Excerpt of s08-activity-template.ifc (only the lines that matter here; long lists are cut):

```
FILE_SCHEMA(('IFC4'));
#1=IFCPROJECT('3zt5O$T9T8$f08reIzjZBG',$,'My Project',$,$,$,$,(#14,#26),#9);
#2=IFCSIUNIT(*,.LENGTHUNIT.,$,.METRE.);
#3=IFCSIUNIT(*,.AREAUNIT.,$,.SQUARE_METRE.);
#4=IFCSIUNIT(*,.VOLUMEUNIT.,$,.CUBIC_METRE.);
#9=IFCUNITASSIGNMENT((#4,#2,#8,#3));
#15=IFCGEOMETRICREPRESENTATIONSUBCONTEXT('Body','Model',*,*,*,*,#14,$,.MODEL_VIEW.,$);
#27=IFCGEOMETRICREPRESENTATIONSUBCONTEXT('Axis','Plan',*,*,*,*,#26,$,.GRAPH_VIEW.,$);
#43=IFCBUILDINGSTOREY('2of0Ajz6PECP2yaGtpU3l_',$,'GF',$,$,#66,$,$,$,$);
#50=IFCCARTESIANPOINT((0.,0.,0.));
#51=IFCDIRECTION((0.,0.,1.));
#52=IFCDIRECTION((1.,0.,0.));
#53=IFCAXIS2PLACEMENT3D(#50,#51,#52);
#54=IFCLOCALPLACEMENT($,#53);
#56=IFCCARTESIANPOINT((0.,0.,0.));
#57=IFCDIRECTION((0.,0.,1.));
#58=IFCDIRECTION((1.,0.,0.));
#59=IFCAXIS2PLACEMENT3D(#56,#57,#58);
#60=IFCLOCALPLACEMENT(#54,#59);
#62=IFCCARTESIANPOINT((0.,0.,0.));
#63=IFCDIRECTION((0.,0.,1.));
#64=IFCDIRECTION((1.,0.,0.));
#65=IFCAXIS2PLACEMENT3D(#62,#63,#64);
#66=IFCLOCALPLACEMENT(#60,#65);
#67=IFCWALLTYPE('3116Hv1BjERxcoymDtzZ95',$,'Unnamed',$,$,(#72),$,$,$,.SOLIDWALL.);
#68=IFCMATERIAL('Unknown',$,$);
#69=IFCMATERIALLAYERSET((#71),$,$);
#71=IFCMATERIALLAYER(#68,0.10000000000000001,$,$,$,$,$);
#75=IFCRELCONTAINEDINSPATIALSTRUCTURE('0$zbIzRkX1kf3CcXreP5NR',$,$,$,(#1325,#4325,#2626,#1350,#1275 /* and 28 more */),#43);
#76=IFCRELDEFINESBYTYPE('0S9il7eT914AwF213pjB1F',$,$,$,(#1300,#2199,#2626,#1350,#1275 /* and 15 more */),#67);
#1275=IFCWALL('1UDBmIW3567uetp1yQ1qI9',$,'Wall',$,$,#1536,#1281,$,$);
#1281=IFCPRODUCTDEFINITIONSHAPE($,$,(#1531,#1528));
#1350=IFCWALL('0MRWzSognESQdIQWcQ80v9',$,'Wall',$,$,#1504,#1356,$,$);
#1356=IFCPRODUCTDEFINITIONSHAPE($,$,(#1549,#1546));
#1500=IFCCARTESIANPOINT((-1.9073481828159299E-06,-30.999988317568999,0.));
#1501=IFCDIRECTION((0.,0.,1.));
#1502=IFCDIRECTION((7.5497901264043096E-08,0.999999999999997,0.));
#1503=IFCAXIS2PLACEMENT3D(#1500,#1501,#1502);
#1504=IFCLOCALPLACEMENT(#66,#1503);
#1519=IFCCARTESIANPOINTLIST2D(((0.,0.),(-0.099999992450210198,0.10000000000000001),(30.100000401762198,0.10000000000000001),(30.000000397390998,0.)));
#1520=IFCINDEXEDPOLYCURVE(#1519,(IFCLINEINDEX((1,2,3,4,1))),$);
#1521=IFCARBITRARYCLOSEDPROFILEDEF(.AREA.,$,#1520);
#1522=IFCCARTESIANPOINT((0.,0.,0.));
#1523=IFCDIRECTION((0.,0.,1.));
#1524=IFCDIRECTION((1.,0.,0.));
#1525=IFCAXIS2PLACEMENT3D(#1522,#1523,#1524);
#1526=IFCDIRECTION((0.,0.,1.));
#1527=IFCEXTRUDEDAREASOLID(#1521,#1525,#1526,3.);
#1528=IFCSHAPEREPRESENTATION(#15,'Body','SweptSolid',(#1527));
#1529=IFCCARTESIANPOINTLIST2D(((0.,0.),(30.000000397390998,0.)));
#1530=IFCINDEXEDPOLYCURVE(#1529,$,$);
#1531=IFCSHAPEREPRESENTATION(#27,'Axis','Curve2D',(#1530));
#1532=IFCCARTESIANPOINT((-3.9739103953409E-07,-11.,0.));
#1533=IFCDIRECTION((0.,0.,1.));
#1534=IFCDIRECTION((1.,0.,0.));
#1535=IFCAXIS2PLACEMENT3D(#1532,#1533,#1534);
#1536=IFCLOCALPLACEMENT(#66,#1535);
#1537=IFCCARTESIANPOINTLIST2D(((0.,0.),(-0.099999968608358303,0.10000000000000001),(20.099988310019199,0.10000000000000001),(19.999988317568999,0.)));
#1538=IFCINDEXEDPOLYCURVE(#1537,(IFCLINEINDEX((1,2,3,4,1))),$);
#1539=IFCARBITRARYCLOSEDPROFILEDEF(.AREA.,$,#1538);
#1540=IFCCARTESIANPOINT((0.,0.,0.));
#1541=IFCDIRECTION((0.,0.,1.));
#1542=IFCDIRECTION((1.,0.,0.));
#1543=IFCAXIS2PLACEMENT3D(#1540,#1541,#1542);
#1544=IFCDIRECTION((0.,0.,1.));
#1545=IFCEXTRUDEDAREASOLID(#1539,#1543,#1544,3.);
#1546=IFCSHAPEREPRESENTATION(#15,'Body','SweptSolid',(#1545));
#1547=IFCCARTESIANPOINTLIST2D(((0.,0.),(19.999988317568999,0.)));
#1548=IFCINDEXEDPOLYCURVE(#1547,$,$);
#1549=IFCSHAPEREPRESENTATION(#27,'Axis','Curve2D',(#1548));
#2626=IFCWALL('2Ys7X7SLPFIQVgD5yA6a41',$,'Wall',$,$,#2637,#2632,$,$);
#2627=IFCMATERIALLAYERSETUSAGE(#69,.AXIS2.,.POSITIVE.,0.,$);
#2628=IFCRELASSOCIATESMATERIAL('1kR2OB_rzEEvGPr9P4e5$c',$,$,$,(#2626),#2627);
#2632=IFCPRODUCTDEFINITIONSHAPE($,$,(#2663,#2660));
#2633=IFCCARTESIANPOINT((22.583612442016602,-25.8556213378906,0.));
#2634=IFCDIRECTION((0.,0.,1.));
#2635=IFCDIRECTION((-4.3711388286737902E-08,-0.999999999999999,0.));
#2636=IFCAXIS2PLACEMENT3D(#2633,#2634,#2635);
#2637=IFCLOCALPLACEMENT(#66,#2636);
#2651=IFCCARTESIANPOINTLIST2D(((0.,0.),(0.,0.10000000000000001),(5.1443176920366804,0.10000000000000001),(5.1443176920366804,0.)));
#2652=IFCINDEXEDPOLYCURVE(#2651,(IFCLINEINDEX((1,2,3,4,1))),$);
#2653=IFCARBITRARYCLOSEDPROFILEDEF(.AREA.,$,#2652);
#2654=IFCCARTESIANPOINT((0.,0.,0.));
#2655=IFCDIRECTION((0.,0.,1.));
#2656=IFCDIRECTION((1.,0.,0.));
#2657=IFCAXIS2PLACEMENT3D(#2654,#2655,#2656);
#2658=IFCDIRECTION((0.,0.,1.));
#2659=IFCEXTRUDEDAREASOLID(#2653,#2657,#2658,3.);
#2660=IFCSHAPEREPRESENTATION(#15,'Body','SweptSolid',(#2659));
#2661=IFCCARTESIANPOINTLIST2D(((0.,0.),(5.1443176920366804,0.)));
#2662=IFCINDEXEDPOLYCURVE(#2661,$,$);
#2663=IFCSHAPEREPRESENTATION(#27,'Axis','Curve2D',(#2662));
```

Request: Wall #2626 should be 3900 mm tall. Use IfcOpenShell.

```python
import ifcopenshell
import ifcopenshell.geom
import ifcopenshell.util.representation
import ifcopenshell.util.shape

model = ifcopenshell.open("s08-activity-template.ifc")
settings = ifcopenshell.geom.settings()


def volume(element):
    """Net volume in cubic metres, openings subtracted."""
    shape = ifcopenshell.geom.create_shape(settings, element)
    return ifcopenshell.util.shape.get_volume(shape.geometry)


wall = model.by_guid("2Ys7X7SLPFIQVgD5yA6a41")
before = volume(wall)

body = ifcopenshell.util.representation.get_representation(wall, "Model", "Body")
solid = body.Items[0]
old_height = solid.Depth
solid.Depth = 3.9
after = volume(wall)

print(f"height {old_height:g} -> {solid.Depth:g}, volume {before:.3f} -> {after:.3f} m3")

model.write("s08-activity-template_edited.ifc")
```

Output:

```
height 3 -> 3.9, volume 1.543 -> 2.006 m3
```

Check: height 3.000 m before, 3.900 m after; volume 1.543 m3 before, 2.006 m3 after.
